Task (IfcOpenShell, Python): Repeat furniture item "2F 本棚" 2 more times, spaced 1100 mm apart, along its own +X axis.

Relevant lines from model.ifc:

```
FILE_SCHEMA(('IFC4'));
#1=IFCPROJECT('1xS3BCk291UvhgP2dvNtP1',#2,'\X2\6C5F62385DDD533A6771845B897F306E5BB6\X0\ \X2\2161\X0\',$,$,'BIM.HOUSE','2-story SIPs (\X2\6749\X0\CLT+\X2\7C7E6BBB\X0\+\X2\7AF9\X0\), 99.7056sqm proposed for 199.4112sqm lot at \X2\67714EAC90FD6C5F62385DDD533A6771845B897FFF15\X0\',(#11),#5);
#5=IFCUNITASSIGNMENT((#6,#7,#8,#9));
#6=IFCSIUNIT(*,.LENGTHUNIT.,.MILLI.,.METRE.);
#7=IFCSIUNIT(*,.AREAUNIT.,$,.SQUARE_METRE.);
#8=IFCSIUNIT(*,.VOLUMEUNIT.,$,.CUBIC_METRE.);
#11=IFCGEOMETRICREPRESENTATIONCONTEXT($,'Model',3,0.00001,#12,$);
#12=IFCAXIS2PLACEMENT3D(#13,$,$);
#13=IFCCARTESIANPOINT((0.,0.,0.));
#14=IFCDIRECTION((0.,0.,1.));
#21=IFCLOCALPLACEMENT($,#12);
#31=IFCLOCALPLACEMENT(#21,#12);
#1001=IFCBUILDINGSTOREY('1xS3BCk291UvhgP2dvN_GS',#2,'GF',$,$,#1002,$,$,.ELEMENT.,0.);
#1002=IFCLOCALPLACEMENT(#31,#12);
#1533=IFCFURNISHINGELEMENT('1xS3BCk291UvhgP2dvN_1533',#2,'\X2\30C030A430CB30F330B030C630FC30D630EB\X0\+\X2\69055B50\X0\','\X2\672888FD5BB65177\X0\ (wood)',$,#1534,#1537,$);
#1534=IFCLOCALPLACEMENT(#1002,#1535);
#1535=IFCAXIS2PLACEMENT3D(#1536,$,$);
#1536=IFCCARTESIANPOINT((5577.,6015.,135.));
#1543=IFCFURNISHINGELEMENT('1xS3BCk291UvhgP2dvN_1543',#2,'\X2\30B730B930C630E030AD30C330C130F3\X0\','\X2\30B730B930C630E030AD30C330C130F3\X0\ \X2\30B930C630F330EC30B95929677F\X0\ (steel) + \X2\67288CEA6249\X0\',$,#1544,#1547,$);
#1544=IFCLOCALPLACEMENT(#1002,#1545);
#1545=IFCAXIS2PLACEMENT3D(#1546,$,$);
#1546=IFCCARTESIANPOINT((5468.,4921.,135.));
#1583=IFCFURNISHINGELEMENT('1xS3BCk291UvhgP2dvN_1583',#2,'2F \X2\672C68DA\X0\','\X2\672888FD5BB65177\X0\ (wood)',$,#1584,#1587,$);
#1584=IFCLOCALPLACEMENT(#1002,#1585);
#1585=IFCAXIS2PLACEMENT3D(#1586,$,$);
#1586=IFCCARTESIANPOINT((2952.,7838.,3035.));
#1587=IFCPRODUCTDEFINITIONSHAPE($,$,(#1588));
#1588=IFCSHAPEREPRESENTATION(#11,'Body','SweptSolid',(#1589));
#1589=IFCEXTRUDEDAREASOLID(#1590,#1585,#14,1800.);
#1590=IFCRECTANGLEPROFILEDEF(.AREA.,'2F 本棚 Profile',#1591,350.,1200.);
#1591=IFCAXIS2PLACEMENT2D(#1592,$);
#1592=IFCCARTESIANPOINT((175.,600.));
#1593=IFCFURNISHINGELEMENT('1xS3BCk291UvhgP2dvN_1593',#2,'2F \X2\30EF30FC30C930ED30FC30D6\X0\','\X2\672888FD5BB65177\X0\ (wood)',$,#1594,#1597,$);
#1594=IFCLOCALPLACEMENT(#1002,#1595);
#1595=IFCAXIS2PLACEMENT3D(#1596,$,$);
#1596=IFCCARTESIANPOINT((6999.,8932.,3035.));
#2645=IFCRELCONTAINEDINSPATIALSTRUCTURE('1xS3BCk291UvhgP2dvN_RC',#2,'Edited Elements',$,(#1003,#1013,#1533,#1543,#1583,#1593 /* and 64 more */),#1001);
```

```python
import ifcopenshell
import ifcopenshell.api.geometry
import ifcopenshell.api.root
import ifcopenshell.util.element
import ifcopenshell.util.placement
import ifcopenshell.util.unit

model = ifcopenshell.open("model.ifc")
unit_scale = ifcopenshell.util.unit.calculate_unit_scale(model)


def reuse_history(source, copy):
    """copy_class also copies each property set's owner history, people and application; keep the originals."""
    for rel in copy.IsDefinedBy:
        if rel.is_a("IfcRelDefinesByProperties") and (history := rel.RelatingPropertyDefinition.OwnerHistory):
            rel.RelatingPropertyDefinition.OwnerHistory = source.OwnerHistory
            ifcopenshell.util.element.remove_deep2(model, history)


source = model.by_id(1583)
base = ifcopenshell.util.placement.get_local_placement(source.ObjectPlacement)
step = base[:3, 0] * 1.1 / unit_scale

for i in range(1, 3):
    copy = ifcopenshell.api.root.copy_class(model, product=source)
    copy.Representation = ifcopenshell.util.element.copy_deep(
        model, source.Representation, exclude=["IfcGeometricRepresentationContext", "IfcRepresentationMap"]
    )
    reuse_history(source, copy)
    matrix = base.copy()
    matrix[:3, 3] += i * step
    print("added at", matrix[:3, 3].round(3) + 0.0)
    ifcopenshell.api.geometry.edit_object_placement(model, product=copy, matrix=matrix, is_si=False)

model.write("model_updated.ifc")
```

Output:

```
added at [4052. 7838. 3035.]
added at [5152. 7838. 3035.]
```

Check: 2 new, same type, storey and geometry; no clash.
